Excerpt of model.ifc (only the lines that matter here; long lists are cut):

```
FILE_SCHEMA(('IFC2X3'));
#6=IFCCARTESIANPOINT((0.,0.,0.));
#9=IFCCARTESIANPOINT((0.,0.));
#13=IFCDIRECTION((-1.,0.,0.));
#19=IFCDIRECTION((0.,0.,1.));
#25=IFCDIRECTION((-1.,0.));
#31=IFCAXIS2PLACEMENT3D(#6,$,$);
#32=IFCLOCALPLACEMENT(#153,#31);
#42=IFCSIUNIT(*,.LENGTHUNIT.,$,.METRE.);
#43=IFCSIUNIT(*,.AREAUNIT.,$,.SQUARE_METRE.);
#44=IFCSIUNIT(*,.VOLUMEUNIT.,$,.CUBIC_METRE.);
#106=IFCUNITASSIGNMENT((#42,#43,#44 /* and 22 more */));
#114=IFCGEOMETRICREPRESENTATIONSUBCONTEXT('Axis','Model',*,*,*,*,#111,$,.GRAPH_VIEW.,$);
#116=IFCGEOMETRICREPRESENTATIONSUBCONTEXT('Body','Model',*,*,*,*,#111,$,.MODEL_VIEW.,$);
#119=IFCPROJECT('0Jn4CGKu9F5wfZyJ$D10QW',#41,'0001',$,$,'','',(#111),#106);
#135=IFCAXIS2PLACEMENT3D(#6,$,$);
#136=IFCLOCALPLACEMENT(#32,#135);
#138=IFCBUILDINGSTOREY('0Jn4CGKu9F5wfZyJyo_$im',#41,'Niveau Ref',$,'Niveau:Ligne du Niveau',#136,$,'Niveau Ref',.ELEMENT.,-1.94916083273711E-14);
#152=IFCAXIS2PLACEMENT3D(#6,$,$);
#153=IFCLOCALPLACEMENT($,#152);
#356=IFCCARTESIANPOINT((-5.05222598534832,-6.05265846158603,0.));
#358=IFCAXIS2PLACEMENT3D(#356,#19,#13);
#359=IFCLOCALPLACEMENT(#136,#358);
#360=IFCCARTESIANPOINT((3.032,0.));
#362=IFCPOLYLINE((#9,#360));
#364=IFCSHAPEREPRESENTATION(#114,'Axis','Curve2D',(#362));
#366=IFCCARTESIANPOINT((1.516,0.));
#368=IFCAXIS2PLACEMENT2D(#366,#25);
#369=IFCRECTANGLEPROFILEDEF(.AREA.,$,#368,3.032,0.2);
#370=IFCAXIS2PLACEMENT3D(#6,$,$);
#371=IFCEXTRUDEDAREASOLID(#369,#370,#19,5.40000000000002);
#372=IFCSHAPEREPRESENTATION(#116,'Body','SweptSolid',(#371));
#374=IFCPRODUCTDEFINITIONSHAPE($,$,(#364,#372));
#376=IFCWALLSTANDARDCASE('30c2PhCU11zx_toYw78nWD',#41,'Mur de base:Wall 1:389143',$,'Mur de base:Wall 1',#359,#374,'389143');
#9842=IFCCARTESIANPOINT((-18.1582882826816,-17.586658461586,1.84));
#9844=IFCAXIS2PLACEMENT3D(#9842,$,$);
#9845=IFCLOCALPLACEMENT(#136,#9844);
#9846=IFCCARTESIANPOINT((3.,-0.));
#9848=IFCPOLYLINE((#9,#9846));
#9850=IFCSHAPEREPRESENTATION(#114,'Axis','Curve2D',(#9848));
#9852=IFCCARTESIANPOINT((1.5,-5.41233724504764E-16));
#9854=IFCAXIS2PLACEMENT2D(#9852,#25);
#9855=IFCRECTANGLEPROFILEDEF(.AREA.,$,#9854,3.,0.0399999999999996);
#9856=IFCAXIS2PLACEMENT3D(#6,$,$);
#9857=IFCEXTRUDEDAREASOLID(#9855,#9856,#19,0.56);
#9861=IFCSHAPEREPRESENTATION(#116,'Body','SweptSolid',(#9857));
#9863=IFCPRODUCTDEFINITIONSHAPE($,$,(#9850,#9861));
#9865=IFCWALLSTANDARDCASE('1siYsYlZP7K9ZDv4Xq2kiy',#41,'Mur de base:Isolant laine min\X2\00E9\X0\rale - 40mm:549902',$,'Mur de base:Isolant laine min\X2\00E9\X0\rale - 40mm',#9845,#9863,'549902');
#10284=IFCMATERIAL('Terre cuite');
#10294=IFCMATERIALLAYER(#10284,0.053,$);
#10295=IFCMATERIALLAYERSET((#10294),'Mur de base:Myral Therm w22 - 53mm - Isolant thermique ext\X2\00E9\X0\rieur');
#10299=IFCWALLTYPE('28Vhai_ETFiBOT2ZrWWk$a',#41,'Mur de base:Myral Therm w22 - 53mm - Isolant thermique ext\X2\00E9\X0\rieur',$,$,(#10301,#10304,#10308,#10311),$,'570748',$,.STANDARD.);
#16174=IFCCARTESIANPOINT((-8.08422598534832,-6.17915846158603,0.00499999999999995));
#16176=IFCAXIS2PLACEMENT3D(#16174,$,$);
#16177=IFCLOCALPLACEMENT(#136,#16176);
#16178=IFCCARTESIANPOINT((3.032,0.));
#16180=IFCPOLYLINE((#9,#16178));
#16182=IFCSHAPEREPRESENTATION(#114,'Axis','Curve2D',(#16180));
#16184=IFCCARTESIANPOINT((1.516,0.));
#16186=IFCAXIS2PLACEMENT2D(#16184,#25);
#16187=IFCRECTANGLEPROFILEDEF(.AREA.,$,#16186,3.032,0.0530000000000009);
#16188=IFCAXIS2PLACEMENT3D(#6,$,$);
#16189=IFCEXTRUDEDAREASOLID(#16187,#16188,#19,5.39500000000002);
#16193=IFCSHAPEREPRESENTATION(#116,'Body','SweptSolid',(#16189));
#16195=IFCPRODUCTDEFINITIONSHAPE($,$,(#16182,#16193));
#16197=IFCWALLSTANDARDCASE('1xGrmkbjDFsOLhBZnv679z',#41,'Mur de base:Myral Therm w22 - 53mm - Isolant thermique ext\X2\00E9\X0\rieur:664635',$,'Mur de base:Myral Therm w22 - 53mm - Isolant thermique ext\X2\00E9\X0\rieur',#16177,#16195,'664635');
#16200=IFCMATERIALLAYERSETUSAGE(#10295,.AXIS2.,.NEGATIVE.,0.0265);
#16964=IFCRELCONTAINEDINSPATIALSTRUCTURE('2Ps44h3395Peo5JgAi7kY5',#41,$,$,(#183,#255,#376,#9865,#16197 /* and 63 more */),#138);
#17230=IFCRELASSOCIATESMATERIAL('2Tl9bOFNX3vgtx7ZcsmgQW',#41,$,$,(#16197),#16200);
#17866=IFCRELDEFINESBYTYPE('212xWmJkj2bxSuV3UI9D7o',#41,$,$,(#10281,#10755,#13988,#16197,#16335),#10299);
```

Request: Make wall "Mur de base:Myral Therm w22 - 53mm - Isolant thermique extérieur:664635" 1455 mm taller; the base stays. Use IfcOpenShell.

```python
import ifcopenshell
import ifcopenshell.geom
import ifcopenshell.util.representation
import ifcopenshell.util.shape
import ifcopenshell.util.unit

model = ifcopenshell.open("model.ifc")
unit_scale = ifcopenshell.util.unit.calculate_unit_scale(model)
settings = ifcopenshell.geom.settings()


def volume(element):
    """Net volume in cubic metres, openings subtracted."""
    shape = ifcopenshell.geom.create_shape(settings, element)
    return ifcopenshell.util.shape.get_volume(shape.geometry)


wall = model.by_guid("1xGrmkbjDFsOLhBZnv679z")
before = volume(wall)

body = ifcopenshell.util.representation.get_representation(wall, "Model", "Body")
solid = body.Items[0]
old_height = solid.Depth
solid.Depth += 1.455 / unit_scale
after = volume(wall)

print(f"height {old_height:g} -> {solid.Depth:g}, volume {before:.3f} -> {after:.3f} m3")

model.write("model-out.ifc")
```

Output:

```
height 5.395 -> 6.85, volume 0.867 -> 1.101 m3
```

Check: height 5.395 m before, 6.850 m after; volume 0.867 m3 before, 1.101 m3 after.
